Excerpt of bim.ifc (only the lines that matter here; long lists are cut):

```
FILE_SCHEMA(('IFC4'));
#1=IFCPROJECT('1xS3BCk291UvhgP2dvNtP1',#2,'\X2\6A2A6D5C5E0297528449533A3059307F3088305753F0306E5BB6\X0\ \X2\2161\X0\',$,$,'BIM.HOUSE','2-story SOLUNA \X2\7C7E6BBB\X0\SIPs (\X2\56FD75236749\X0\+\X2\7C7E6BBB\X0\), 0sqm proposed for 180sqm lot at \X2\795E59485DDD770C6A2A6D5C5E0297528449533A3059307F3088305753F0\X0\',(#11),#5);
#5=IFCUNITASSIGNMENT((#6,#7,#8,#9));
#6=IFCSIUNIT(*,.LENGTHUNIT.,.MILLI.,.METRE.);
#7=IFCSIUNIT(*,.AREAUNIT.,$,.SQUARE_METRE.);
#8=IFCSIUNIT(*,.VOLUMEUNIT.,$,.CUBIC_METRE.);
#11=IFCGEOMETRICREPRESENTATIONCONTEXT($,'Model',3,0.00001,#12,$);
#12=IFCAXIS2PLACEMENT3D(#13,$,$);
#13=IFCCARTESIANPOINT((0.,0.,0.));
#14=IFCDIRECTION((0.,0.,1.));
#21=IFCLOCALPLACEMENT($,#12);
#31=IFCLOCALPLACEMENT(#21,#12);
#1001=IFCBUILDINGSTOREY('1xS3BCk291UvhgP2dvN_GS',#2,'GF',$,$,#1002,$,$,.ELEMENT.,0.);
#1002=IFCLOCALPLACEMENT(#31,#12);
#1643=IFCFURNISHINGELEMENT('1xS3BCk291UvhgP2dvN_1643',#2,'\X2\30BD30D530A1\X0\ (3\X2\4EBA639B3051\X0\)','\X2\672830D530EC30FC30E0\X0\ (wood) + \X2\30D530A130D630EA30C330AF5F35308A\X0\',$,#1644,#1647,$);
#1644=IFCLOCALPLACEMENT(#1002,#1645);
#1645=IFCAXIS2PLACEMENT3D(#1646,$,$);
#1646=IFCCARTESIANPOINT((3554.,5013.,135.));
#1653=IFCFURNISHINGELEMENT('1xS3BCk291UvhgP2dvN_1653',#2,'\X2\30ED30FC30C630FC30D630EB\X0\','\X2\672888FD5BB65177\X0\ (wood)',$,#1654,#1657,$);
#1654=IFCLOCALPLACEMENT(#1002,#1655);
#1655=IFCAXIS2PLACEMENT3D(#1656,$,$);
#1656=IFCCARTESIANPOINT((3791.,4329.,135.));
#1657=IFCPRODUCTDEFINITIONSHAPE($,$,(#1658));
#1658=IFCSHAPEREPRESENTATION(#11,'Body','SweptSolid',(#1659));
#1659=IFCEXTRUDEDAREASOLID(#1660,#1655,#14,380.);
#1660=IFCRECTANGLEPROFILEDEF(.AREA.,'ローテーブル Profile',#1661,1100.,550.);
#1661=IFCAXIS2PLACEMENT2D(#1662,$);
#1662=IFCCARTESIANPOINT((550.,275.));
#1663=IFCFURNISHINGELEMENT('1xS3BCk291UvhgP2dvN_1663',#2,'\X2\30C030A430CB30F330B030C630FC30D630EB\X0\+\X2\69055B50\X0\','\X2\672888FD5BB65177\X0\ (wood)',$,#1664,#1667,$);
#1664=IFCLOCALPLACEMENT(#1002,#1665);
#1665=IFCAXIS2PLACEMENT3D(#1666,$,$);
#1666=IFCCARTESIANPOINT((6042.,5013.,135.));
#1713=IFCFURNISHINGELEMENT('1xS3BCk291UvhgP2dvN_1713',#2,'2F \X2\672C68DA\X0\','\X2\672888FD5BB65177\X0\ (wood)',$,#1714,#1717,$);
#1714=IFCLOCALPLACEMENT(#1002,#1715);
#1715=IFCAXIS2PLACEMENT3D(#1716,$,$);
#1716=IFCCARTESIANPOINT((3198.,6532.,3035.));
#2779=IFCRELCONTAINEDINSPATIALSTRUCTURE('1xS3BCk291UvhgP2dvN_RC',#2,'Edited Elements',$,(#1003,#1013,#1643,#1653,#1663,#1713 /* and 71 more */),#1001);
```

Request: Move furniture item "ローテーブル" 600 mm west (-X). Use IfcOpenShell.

```python
import ifcopenshell
import ifcopenshell.api.geometry
import ifcopenshell.util.placement
import ifcopenshell.util.unit

model = ifcopenshell.open("bim.ifc")
unit_scale = ifcopenshell.util.unit.calculate_unit_scale(model)

item = model.by_guid("1xS3BCk291UvhgP2dvN_1653")
matrix = ifcopenshell.util.placement.get_local_placement(item.ObjectPlacement)
matrix[0, 3] -= 0.6 / unit_scale
ifcopenshell.api.geometry.edit_object_placement(model, product=item, matrix=matrix, is_si=False)

print(ifcopenshell.util.placement.get_local_placement(item.ObjectPlacement).round(3) + 0.0)

model.write("bim_v2.ifc")
```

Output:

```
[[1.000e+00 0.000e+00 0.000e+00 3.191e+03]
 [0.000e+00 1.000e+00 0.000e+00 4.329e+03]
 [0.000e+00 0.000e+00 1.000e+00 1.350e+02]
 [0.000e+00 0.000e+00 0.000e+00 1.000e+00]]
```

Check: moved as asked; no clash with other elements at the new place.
